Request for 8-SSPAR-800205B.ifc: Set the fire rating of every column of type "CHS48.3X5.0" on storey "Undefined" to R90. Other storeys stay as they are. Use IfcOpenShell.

First a look at what the model holds.

```python
import ifcopenshell
import ifcopenshell.util.element

model = ifcopenshell.open("8-SSPAR-800205B.ifc")
print(model.schema)
storey = next(s for s in model.by_type("IfcBuildingStorey") if s.Name == "Undefined")
columns = [e for e in ifcopenshell.util.element.get_decomposition(storey) if e.is_a("IfcColumn")]
seen = {}
for e in columns:
    element_type = ifcopenshell.util.element.get_type(e)
    key = (element_type.Name if element_type != e and element_type else None, ifcopenshell.util.element.get_pset(e, "Pset_ColumnCommon", "FireRating"))
    seen[key] = seen.get(key, 0) + 1
for (name, value), count in sorted(seen.items(), key=str):
    print(count, "x", name, "|", value)
```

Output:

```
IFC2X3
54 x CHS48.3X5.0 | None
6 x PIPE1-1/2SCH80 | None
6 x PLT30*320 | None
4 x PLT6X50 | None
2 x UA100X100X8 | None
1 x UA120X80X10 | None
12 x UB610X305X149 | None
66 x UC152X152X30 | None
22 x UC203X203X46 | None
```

```python
import ifcopenshell
import ifcopenshell.api.pset
import ifcopenshell.util.element

model = ifcopenshell.open("8-SSPAR-800205B.ifc")

storey = next(s for s in model.by_type("IfcBuildingStorey") if s.Name == "Undefined")
columns = [e for e in ifcopenshell.util.element.get_decomposition(storey) if e.is_a("IfcColumn")]

count = 0
for e in columns:
    element_type = ifcopenshell.util.element.get_type(e)
    if element_type in (None, e) or element_type.Name != "CHS48.3X5.0":
        continue
    # add_pset returns the element's existing set when there is one.
    pset = ifcopenshell.api.pset.add_pset(model, product=e, name="Pset_ColumnCommon")
    ifcopenshell.api.pset.edit_pset(model, pset=pset, properties={"FireRating": "R90"})
    count += 1

print(count, "columns updated")

model.write("8-SSPAR-800205B-out.ifc")
```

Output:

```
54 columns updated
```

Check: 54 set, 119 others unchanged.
